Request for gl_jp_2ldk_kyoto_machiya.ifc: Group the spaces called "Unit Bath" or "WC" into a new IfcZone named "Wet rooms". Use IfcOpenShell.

First a look at what the model holds.

```python
import ifcopenshell

model = ifcopenshell.open("gl_jp_2ldk_kyoto_machiya.ifc")
print(model.schema)
seen = {}
for space in model.by_type("IfcSpace"):
    seen[space.LongName] = seen.get(space.LongName, 0) + 1
for name, count in sorted(seen.items(), key=str):
    print(count, "x", name)
print("zones:", [z.Name for z in model.by_type("IfcZone")][:20])
```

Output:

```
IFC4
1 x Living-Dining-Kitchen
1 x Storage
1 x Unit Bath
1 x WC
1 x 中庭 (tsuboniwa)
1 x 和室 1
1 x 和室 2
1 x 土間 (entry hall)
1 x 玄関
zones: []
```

```python
import ifcopenshell
import ifcopenshell.api.group
import ifcopenshell.api.root

model = ifcopenshell.open("gl_jp_2ldk_kyoto_machiya.ifc")

names = {"Unit Bath", "WC"}
spaces = [s for s in model.by_type("IfcSpace") if s.LongName in names]

zone = ifcopenshell.api.root.create_entity(model, ifc_class="IfcZone", name="Wet rooms")
ifcopenshell.api.group.assign_group(model, products=spaces, group=zone)
print(len(spaces), "spaces in", zone.Name)

model.write("gl_jp_2ldk_kyoto_machiya_rev.ifc")
```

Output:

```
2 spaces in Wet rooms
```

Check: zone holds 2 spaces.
